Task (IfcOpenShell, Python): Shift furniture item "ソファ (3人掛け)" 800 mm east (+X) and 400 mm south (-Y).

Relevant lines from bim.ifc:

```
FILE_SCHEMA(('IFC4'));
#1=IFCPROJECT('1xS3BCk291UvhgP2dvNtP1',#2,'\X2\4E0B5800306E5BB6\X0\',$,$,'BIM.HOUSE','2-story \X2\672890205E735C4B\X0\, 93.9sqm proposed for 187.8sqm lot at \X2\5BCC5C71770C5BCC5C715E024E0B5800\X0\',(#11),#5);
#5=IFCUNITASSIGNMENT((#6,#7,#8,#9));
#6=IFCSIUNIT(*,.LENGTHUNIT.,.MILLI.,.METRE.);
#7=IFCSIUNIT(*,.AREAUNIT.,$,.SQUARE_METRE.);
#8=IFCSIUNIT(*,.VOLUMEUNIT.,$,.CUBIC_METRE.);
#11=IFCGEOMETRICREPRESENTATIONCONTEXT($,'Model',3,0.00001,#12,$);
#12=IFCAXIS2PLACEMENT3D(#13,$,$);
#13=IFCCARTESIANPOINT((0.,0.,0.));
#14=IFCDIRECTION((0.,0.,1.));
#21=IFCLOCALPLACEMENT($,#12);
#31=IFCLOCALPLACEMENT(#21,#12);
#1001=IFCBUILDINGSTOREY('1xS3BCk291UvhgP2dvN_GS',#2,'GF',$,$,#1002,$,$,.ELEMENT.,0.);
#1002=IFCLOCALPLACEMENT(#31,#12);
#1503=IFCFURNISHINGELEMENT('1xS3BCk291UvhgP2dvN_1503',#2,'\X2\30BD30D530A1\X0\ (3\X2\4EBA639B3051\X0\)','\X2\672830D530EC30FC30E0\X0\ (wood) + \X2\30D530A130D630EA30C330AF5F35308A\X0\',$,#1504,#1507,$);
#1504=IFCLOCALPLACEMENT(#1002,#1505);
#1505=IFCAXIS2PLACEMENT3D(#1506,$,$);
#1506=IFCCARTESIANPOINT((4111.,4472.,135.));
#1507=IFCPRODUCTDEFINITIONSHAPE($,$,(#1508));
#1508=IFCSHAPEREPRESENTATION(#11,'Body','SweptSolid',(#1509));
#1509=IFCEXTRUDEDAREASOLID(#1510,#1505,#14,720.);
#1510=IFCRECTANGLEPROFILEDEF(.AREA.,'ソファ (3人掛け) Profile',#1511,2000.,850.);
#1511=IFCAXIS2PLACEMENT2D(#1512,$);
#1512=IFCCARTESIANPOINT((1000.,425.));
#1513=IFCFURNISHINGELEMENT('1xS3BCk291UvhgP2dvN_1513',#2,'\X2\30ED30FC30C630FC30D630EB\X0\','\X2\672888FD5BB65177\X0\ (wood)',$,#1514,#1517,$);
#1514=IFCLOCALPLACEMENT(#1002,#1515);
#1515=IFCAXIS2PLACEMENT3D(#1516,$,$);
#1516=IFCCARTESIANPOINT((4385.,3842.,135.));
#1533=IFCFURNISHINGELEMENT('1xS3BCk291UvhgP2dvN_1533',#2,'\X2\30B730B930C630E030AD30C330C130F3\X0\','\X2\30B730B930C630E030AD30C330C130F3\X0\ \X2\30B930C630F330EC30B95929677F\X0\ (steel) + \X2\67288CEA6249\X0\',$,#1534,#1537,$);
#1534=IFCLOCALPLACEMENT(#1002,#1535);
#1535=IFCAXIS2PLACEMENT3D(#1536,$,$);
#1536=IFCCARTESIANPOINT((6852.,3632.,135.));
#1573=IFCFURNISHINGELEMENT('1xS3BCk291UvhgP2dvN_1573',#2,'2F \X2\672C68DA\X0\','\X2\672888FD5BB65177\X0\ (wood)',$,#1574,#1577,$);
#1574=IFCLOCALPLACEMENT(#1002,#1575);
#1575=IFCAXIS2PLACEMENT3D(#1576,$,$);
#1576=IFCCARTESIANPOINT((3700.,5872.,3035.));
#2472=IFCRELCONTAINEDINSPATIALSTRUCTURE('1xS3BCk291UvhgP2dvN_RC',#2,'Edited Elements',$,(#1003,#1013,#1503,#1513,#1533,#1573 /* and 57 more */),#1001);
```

```python
import ifcopenshell
import ifcopenshell.api.geometry
import ifcopenshell.util.placement
import ifcopenshell.util.unit

model = ifcopenshell.open("bim.ifc")
unit_scale = ifcopenshell.util.unit.calculate_unit_scale(model)

item = model.by_id(1503)
matrix = ifcopenshell.util.placement.get_local_placement(item.ObjectPlacement)
matrix[0, 3] += 0.8 / unit_scale
matrix[1, 3] -= 0.4 / unit_scale
ifcopenshell.api.geometry.edit_object_placement(model, product=item, matrix=matrix, is_si=False)

print(ifcopenshell.util.placement.get_local_placement(item.ObjectPlacement).round(3) + 0.0)

model.write("bim_edited.ifc")
```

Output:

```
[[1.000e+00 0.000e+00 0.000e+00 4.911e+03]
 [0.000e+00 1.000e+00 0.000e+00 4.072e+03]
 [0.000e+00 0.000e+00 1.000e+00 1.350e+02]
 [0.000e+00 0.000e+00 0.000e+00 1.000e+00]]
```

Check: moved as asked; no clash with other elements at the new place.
